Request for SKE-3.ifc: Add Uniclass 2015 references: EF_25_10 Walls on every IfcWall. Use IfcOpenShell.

First a look at what the model holds.

```python
import ifcopenshell

model = ifcopenshell.open("SKE-3.ifc")
print(model.schema)
print("classifications:", [c.Name for c in model.by_type("IfcClassification")])
for ifc_class in ("IfcDoor", "IfcRoof", "IfcStair", "IfcWall", "IfcWindow"):
    print(ifc_class, len(model.by_type(ifc_class)))
```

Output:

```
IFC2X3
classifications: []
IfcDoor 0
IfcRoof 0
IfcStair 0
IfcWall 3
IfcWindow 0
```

```python
import ifcopenshell
import ifcopenshell.api.classification

model = ifcopenshell.open("SKE-3.ifc")

# IFC2X3 requires Source and Edition and has no link from the project to the system.
system = model.create_entity("IfcClassification", Source="NBS", Edition="2015", Name="Uniclass 2015")

codes = {
    "IfcWall": ("EF_25_10", "Walls"),
}
for ifc_class, (code, name) in codes.items():
    products = model.by_type(ifc_class)
    ifcopenshell.api.classification.add_reference(
        model, products=products, classification=system, identification=code, name=name
    )
    print(code, len(products))

model.write("SKE-3_updated.ifc")
```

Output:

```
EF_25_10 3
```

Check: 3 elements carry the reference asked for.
